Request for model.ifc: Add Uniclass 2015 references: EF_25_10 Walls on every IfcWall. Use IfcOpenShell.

First a look at what the model holds.

```python
import ifcopenshell

model = ifcopenshell.open("model.ifc")
print(model.schema)
print("classifications:", [c.Name for c in model.by_type("IfcClassification")])
for ifc_class in ("IfcDoor", "IfcRoof", "IfcStair", "IfcWall", "IfcWindow"):
    print(ifc_class, len(model.by_type(ifc_class)))
```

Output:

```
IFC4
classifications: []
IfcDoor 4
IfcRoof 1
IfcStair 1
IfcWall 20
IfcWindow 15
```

```python
import ifcopenshell
import ifcopenshell.api.classification

model = ifcopenshell.open("model.ifc")

system = ifcopenshell.api.classification.add_classification(model, classification="Uniclass 2015")

codes = {
    "IfcWall": ("EF_25_10", "Walls"),
}
for ifc_class, (code, name) in codes.items():
    products = model.by_type(ifc_class)
    ifcopenshell.api.classification.add_reference(
        model, products=products, classification=system, identification=code, name=name
    )
    print(code, len(products))

model.write("model_rev.ifc")
```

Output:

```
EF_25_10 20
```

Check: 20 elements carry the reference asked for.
